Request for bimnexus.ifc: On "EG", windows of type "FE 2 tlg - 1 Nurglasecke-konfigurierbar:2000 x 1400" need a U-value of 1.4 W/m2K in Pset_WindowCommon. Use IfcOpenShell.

First a look at what the model holds.

```python
import ifcopenshell
import ifcopenshell.util.element

model = ifcopenshell.open("bimnexus.ifc")
print(model.schema)
storey = next(s for s in model.by_type("IfcBuildingStorey") if s.Name == "EG")
windows = [e for e in ifcopenshell.util.element.get_decomposition(storey) if e.is_a("IfcWindow")]
seen = {}
for e in windows:
    element_type = ifcopenshell.util.element.get_type(e)
    key = (element_type.Name if element_type != e and element_type else None, ifcopenshell.util.element.get_pset(e, "Pset_WindowCommon", "ThermalTransmittance"))
    seen[key] = seen.get(key, 0) + 1
for (name, value), count in sorted(seen.items(), key=str):
    print(count, "x", name, "|", value)
```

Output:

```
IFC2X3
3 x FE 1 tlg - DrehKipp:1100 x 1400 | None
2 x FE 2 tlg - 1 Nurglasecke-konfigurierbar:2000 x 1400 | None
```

```python
import ifcopenshell
import ifcopenshell.api.pset
import ifcopenshell.util.element

model = ifcopenshell.open("bimnexus.ifc")

storey = next(s for s in model.by_type("IfcBuildingStorey") if s.Name == "EG")
windows = [e for e in ifcopenshell.util.element.get_decomposition(storey) if e.is_a("IfcWindow")]

count = 0
for e in windows:
    element_type = ifcopenshell.util.element.get_type(e)
    if element_type in (None, e) or element_type.Name != "FE 2 tlg - 1 Nurglasecke-konfigurierbar:2000 x 1400":
        continue
    # add_pset returns the element's existing set when there is one.
    pset = ifcopenshell.api.pset.add_pset(model, product=e, name="Pset_WindowCommon")
    ifcopenshell.api.pset.edit_pset(model, pset=pset, properties={"ThermalTransmittance": 1.4})
    count += 1

print(count, "windows updated")

model.write("bimnexus_rev.ifc")
```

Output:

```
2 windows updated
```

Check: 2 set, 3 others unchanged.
